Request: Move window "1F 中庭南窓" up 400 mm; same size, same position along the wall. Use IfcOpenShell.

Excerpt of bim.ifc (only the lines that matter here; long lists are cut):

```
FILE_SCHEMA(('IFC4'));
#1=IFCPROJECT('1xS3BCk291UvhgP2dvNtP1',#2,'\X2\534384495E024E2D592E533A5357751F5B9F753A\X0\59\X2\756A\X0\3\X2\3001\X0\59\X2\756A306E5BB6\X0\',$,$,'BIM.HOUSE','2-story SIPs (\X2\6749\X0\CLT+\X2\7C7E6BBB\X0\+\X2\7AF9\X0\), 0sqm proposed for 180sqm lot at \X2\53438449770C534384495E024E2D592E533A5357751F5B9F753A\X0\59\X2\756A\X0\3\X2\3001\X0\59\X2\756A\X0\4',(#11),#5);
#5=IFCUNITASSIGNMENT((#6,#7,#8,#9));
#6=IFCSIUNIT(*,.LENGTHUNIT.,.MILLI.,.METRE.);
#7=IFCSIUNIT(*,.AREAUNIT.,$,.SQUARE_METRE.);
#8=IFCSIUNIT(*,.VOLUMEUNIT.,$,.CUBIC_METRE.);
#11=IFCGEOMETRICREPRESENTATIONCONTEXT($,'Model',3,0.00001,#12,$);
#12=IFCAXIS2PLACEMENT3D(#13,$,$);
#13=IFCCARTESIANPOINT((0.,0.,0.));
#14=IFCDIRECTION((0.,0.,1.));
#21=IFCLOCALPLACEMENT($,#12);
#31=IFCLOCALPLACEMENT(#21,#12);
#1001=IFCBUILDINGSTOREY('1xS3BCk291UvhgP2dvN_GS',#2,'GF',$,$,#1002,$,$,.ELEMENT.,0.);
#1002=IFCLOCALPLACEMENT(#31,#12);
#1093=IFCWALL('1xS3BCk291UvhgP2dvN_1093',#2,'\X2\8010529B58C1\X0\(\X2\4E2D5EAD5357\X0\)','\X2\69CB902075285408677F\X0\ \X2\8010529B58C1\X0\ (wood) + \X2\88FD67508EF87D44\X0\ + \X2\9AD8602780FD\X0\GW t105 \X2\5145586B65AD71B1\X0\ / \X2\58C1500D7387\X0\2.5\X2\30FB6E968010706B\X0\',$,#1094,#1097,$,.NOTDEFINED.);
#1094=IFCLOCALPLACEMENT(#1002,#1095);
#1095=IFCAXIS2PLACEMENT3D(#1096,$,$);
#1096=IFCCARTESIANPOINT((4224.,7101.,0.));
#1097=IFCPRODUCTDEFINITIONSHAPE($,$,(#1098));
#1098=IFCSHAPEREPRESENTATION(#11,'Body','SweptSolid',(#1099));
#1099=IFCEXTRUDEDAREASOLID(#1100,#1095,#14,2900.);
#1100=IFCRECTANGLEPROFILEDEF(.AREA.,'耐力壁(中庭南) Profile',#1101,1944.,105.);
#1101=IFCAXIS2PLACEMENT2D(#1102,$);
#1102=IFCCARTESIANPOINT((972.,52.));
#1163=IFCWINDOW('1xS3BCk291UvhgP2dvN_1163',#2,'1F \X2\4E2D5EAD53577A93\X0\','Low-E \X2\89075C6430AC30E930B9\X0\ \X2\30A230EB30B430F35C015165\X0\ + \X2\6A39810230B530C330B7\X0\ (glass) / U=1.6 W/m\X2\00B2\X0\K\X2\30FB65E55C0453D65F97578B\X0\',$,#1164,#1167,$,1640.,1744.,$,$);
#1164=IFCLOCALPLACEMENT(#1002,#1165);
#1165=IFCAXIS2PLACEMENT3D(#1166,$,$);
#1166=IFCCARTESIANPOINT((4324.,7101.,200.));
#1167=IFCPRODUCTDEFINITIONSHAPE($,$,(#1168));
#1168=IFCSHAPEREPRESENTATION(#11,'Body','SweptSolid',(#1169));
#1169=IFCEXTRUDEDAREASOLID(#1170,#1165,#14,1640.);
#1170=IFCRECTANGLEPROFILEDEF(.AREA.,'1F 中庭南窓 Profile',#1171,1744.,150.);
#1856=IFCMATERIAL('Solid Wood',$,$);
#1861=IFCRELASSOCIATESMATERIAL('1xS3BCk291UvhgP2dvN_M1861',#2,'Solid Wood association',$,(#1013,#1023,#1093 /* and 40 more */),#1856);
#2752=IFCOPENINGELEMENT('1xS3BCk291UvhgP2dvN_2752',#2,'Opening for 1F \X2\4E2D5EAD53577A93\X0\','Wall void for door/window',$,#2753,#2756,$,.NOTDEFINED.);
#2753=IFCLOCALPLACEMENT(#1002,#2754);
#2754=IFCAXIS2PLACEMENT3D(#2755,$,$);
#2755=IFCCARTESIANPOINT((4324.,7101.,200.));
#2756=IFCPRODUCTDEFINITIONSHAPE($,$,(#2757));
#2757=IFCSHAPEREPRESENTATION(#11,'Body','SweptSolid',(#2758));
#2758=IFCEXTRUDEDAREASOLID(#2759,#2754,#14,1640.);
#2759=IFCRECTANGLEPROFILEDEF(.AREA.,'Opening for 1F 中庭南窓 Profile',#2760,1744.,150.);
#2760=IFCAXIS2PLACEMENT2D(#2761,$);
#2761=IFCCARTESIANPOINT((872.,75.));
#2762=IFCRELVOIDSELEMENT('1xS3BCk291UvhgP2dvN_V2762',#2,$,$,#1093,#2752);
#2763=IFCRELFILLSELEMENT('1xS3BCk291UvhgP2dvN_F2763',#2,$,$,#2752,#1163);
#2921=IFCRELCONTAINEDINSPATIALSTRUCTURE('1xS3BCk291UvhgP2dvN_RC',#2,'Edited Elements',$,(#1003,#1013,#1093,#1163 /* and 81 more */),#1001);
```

```python
import numpy as np
import ifcopenshell
import ifcopenshell.api.geometry
import ifcopenshell.util.placement
import ifcopenshell.util.unit

model = ifcopenshell.open("bim.ifc")
unit_scale = ifcopenshell.util.unit.calculate_unit_scale(model)

window = model.by_guid("1xS3BCk291UvhgP2dvN_1163")
opening = window.FillsVoids[0].RelatingOpeningElement
dz = 0.4 / unit_scale

shift = np.array([0.0, 0.0, dz])
# The window is not placed relative to its opening, so move both.
for product in (opening, window):
    matrix = ifcopenshell.util.placement.get_local_placement(product.ObjectPlacement)
    matrix[:3, 3] += shift
    ifcopenshell.api.geometry.edit_object_placement(model, product=product, matrix=matrix, is_si=False)

print(f"moved by {dz * unit_scale:+.3f} m")

model.write("bim_v2.ifc")
```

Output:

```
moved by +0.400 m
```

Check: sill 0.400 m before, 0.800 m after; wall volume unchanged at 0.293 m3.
